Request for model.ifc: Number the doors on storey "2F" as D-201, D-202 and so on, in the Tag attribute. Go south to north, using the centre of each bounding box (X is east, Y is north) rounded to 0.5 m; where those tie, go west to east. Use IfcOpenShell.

First a look at what the model holds.

```python
import ifcopenshell
import ifcopenshell.util.element
import ifcopenshell.util.placement

model = ifcopenshell.open("model.ifc")
print(model.schema)
storey = next(s for s in model.by_type("IfcBuildingStorey") if s.Name == "2F")
doors = [e for e in ifcopenshell.util.element.get_decomposition(storey) if e.is_a("IfcDoor")]
for e in sorted(doors, key=lambda e: e.id()):
    origin = ifcopenshell.util.placement.get_local_placement(e.ObjectPlacement)[:3, 3]
    print(e.id(), e.Tag, e.Name, origin.round(2) + 0.0, sep=" | ")
```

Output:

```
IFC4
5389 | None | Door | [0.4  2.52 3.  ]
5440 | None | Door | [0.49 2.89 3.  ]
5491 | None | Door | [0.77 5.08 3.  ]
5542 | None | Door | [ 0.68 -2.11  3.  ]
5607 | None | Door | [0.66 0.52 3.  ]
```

```python
import ifcopenshell
import ifcopenshell.geom
import ifcopenshell.util.element
import ifcopenshell.util.shape

model = ifcopenshell.open("model.ifc")
settings = ifcopenshell.geom.settings()
settings.set("use-world-coords", True)


def centre(element):
    shape = ifcopenshell.geom.create_shape(settings, element)
    return ifcopenshell.util.shape.get_bbox_centroid(shape.geometry)


storey = next(s for s in model.by_type("IfcBuildingStorey") if s.Name == "2F")
doors = [e for e in ifcopenshell.util.element.get_decomposition(storey) if e.is_a("IfcDoor")]

# Insertion points can sit at a corner or the storey origin, so sort by the geometry (in metres).
centres = {e: centre(e) for e in doors}
doors.sort(key=lambda e: (round(centres[e][1] / 0.5), centres[e][0]))

for i, e in enumerate(doors, start=1):
    number = f"D-2{i:02d}"
    e.Tag = number
    print(e.id(), number)

model.write("model_edited.ifc")
```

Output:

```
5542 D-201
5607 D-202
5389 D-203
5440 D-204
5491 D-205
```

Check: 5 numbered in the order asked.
